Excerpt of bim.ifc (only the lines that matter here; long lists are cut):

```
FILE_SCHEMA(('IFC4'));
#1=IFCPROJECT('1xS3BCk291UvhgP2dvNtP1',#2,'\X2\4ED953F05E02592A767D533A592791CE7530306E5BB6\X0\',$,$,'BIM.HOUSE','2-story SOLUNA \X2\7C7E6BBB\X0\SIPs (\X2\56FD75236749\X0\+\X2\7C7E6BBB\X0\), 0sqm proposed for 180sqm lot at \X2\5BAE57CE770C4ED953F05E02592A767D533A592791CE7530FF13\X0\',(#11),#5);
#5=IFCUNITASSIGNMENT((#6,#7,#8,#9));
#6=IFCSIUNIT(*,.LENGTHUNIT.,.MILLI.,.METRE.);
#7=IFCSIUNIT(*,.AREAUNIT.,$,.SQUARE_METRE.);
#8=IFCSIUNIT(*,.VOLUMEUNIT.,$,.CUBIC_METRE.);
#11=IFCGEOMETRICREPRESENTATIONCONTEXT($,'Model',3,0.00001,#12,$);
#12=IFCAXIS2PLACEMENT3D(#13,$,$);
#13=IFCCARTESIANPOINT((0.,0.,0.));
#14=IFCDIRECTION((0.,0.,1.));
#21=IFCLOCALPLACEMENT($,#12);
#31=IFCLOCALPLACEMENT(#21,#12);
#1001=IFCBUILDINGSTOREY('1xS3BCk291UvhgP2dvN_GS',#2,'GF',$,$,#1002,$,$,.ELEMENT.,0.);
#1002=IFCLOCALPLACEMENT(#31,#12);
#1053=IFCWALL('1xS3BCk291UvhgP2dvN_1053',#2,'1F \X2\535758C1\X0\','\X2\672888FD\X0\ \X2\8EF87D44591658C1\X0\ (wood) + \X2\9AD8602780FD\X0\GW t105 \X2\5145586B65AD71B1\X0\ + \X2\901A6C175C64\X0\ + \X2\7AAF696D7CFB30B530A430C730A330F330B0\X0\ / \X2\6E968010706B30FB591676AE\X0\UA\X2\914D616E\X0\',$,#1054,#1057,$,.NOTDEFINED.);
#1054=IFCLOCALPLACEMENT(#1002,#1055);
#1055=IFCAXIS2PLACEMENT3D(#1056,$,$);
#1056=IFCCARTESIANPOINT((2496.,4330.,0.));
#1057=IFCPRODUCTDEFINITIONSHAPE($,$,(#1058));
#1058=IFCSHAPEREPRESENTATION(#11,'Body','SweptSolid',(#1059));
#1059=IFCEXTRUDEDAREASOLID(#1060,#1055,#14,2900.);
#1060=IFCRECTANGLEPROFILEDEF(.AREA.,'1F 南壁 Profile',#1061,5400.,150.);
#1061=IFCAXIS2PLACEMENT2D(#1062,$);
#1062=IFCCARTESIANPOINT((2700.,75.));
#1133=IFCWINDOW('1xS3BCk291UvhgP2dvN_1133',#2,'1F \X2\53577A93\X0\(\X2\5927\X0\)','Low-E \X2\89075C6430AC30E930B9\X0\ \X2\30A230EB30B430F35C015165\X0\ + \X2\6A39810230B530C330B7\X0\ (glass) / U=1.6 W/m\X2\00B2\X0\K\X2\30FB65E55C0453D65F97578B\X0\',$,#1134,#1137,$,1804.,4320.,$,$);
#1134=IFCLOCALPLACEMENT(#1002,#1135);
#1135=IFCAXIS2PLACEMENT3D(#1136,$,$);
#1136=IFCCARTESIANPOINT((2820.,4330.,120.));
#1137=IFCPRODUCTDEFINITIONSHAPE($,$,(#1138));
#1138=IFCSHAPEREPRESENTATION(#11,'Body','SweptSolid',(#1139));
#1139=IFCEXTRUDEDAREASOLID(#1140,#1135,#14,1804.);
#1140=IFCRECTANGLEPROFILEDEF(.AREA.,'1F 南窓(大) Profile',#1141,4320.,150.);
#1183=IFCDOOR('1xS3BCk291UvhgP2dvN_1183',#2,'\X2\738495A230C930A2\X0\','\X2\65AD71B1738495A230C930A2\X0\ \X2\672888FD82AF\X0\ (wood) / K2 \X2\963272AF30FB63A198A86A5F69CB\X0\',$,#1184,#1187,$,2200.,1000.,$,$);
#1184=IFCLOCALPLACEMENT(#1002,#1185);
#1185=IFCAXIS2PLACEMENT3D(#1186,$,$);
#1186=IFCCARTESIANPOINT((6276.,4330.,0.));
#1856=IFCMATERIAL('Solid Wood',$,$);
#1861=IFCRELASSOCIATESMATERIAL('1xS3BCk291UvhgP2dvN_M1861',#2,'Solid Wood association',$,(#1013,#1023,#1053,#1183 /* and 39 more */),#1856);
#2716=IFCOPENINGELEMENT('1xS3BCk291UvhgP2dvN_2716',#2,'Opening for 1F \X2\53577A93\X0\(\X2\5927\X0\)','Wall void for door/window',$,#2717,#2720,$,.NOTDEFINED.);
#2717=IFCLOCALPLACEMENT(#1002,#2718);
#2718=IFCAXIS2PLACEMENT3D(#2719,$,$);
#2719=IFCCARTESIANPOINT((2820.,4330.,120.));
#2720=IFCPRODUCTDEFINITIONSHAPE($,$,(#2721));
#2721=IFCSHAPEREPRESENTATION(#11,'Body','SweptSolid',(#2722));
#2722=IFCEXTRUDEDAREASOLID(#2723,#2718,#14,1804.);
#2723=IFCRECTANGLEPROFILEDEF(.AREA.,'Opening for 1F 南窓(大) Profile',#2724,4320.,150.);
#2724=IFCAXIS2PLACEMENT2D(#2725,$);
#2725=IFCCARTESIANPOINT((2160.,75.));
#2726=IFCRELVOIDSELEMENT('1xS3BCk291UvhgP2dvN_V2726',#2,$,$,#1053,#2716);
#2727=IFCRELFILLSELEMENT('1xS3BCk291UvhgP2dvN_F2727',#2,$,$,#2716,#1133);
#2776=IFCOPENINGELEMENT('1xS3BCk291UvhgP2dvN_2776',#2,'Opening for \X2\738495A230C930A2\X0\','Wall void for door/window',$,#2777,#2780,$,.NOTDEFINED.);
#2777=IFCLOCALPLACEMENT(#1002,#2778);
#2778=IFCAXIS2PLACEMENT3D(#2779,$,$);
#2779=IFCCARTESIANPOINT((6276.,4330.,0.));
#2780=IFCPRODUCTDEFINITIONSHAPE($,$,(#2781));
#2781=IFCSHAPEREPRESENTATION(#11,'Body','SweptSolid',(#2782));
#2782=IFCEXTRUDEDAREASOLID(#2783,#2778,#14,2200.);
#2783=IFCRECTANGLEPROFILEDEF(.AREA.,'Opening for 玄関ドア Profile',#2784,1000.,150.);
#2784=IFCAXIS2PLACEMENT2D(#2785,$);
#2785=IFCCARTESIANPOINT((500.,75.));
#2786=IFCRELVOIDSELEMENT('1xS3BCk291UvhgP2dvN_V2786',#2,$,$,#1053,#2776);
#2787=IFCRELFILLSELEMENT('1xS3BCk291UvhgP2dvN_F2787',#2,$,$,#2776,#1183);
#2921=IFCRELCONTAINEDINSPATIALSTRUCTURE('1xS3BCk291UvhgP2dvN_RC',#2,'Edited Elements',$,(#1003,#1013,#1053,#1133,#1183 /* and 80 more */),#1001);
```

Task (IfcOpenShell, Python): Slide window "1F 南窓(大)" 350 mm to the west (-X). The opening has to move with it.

```python
import ifcopenshell
import ifcopenshell.api.geometry
import ifcopenshell.util.placement
import ifcopenshell.util.unit

model = ifcopenshell.open("bim.ifc")
unit_scale = ifcopenshell.util.unit.calculate_unit_scale(model)

window = model.by_guid("1xS3BCk291UvhgP2dvN_1133")
opening = window.FillsVoids[0].RelatingOpeningElement
wall = opening.VoidsElements[0].RelatingBuildingElement

wall_matrix = ifcopenshell.util.placement.get_local_placement(wall.ObjectPlacement)
shift = wall_matrix[:3, 0] * -0.35 / unit_scale
before = ifcopenshell.util.placement.get_local_placement(window.ObjectPlacement)[:3, 3].copy()

# The window is not placed relative to its opening, so move both.
for product in (opening, window):
    matrix = ifcopenshell.util.placement.get_local_placement(product.ObjectPlacement)
    matrix[:3, 3] += shift
    ifcopenshell.api.geometry.edit_object_placement(model, product=product, matrix=matrix, is_si=False)

after = ifcopenshell.util.placement.get_local_placement(window.ObjectPlacement)[:3, 3]
print("window moved by", (after - before).round(3) + 0.0)

model.write("bim-out.ifc")
```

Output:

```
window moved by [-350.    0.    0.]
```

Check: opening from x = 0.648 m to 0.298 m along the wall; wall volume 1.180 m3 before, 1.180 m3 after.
